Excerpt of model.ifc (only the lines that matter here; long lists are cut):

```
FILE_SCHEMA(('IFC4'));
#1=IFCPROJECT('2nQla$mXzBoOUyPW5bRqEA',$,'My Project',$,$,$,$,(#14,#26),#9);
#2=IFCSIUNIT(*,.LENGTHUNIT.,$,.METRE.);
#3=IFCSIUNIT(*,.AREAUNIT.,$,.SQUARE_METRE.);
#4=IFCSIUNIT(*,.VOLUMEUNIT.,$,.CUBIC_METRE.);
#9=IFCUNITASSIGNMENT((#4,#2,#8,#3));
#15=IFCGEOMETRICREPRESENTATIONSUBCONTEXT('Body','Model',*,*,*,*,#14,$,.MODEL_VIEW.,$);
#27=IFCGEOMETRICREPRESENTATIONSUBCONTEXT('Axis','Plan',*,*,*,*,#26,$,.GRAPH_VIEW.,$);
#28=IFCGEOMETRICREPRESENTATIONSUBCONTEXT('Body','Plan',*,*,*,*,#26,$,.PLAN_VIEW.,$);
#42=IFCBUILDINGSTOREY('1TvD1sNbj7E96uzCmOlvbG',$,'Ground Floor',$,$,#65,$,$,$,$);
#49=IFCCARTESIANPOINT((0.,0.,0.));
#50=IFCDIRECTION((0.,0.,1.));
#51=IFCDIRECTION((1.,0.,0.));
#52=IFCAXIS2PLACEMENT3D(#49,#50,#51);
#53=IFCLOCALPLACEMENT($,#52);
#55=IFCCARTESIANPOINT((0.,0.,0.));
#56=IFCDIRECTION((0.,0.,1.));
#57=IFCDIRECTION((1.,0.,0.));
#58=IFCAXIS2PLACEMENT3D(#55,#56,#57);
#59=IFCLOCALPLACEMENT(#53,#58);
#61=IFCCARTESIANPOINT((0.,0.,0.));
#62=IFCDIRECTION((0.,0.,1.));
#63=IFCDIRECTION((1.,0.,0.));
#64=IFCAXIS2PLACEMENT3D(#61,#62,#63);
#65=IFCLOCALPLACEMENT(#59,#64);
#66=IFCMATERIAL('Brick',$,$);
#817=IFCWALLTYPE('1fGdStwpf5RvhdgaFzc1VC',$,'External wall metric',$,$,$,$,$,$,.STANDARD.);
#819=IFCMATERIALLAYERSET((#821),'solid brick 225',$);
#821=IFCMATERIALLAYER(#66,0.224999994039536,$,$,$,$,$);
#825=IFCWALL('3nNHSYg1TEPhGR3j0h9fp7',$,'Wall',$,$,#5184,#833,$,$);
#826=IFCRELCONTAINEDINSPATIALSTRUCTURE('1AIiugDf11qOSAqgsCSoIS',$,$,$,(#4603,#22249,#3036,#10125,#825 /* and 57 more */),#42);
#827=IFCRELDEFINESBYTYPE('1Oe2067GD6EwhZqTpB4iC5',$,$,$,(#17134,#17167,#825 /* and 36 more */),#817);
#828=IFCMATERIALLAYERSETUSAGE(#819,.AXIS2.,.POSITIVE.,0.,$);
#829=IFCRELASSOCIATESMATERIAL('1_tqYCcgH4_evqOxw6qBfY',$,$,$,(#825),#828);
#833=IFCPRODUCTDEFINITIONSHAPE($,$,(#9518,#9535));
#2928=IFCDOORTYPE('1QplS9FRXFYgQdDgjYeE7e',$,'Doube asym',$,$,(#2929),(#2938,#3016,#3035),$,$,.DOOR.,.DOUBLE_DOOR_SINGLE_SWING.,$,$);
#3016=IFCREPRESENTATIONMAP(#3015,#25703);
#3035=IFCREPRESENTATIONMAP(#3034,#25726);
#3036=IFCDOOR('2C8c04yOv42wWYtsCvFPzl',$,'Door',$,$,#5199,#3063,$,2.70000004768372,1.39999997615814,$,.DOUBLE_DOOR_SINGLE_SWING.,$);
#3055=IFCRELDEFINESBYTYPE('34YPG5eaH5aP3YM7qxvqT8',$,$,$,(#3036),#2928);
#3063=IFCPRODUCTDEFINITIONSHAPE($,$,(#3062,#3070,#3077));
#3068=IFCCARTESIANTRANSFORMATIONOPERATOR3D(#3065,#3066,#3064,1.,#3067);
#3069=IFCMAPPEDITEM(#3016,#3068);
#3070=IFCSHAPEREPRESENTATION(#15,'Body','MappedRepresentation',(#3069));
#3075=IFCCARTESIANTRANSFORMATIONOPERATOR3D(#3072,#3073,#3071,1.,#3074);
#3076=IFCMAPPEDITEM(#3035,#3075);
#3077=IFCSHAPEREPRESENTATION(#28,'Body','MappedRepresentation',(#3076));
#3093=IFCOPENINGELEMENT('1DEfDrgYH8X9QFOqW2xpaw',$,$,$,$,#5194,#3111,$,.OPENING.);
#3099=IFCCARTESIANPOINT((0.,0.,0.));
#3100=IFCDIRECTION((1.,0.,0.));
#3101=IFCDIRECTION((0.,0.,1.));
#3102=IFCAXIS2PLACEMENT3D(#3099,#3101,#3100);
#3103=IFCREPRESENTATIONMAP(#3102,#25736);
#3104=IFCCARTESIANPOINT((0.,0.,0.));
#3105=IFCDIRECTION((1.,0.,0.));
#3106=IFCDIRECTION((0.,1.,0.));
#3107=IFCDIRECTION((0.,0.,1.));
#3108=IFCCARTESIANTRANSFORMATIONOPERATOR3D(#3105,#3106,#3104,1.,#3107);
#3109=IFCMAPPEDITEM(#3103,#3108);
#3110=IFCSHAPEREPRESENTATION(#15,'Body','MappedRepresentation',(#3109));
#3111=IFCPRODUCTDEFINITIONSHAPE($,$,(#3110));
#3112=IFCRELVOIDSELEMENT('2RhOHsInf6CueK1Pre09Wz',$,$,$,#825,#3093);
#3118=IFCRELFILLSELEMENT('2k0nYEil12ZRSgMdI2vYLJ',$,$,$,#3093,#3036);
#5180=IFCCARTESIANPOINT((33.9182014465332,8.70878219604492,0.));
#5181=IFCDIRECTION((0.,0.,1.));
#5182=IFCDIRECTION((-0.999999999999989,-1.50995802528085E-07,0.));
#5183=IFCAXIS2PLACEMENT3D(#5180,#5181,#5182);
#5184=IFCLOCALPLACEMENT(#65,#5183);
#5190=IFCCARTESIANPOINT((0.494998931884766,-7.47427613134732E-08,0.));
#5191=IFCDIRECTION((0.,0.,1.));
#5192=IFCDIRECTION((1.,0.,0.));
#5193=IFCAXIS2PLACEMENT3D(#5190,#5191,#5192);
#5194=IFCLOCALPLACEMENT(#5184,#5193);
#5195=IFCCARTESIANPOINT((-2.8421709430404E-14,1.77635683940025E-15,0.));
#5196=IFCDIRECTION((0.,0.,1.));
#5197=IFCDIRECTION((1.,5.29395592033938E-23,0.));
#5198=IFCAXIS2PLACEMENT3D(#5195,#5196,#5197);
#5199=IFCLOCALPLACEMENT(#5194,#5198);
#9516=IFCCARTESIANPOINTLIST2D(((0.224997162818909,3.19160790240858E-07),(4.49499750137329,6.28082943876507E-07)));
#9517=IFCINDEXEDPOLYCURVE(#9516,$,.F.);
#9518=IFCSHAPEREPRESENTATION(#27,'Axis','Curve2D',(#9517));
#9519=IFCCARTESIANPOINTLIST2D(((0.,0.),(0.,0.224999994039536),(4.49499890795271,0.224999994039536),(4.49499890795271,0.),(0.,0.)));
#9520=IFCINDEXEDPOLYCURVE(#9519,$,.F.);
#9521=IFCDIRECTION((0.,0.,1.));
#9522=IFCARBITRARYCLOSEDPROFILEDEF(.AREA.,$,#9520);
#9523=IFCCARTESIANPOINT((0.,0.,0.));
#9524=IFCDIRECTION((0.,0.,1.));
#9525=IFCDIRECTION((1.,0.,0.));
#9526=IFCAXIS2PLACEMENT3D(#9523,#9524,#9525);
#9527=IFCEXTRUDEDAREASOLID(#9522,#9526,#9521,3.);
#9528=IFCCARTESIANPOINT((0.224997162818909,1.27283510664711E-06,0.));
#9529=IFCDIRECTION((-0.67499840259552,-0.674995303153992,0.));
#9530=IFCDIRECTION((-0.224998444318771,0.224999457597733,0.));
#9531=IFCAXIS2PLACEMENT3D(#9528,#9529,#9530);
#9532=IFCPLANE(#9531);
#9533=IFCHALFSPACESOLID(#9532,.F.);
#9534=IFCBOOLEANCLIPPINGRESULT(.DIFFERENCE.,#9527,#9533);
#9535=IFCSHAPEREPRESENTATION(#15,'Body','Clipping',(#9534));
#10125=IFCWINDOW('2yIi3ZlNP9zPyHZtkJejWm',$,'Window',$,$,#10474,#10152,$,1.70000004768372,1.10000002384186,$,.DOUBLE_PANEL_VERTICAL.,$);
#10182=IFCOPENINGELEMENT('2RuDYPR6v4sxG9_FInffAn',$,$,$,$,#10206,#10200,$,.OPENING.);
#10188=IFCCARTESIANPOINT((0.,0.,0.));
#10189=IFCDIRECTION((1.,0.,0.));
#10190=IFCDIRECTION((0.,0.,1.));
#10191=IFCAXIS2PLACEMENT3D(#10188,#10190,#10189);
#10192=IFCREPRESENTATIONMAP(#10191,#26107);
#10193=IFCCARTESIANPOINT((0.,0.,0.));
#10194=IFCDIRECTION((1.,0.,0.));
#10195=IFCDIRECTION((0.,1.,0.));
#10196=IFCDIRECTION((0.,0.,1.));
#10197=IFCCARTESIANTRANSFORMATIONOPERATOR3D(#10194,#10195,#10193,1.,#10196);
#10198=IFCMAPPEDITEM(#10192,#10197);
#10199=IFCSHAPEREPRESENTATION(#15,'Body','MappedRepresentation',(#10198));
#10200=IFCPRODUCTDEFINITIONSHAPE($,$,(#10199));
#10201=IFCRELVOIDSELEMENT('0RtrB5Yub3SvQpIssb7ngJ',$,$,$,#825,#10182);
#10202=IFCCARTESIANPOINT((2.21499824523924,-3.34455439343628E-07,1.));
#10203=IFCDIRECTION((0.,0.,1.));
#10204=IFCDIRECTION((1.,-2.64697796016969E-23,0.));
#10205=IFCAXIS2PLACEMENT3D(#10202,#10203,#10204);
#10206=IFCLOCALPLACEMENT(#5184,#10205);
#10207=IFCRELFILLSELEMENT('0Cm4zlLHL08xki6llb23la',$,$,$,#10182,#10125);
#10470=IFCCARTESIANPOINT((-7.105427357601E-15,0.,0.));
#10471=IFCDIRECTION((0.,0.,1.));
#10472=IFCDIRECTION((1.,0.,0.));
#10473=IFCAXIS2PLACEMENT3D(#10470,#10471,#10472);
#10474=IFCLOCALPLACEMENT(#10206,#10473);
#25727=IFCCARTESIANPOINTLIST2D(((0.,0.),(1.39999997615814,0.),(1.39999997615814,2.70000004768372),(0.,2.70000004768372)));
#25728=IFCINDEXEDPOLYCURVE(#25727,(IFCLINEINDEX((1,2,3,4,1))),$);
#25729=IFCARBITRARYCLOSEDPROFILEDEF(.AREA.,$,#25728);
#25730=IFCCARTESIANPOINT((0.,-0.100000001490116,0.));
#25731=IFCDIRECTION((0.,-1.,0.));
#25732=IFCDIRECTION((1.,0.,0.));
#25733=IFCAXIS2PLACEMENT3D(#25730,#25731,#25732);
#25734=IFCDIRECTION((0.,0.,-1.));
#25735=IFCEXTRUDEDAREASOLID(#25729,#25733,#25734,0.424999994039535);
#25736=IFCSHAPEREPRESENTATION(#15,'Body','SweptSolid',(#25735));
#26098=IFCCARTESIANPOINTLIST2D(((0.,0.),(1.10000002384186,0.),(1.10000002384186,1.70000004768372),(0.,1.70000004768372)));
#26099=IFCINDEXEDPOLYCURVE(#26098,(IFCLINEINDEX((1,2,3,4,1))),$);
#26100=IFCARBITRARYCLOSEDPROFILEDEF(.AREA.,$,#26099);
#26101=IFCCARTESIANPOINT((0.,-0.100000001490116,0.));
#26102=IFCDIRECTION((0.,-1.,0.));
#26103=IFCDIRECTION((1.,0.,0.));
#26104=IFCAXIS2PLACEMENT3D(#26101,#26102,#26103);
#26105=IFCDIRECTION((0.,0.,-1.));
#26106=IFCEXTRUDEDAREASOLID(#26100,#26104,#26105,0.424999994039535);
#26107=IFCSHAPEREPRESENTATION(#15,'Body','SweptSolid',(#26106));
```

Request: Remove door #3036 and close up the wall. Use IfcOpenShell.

```python
import ifcopenshell
import ifcopenshell.api.feature
import ifcopenshell.api.root
import ifcopenshell.geom
import ifcopenshell.util.shape

model = ifcopenshell.open("model.ifc")
settings = ifcopenshell.geom.settings()


def volume(element):
    """Net volume in cubic metres, openings subtracted."""
    shape = ifcopenshell.geom.create_shape(settings, element)
    return ifcopenshell.util.shape.get_volume(shape.geometry)


door = model.by_guid("2C8c04yOv42wWYtsCvFPzl")
opening = door.FillsVoids[0].RelatingOpeningElement
wall = opening.VoidsElements[0].RelatingBuildingElement
before = volume(wall)

ifcopenshell.api.root.remove_product(model, product=door)
ifcopenshell.api.feature.remove_feature(model, feature=opening)

after = volume(wall)

print(f"wall volume {before:.3f} -> {after:.3f} m3")

model.write("model-out.ifc")
```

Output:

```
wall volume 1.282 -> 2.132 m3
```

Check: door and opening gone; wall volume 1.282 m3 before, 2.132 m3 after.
